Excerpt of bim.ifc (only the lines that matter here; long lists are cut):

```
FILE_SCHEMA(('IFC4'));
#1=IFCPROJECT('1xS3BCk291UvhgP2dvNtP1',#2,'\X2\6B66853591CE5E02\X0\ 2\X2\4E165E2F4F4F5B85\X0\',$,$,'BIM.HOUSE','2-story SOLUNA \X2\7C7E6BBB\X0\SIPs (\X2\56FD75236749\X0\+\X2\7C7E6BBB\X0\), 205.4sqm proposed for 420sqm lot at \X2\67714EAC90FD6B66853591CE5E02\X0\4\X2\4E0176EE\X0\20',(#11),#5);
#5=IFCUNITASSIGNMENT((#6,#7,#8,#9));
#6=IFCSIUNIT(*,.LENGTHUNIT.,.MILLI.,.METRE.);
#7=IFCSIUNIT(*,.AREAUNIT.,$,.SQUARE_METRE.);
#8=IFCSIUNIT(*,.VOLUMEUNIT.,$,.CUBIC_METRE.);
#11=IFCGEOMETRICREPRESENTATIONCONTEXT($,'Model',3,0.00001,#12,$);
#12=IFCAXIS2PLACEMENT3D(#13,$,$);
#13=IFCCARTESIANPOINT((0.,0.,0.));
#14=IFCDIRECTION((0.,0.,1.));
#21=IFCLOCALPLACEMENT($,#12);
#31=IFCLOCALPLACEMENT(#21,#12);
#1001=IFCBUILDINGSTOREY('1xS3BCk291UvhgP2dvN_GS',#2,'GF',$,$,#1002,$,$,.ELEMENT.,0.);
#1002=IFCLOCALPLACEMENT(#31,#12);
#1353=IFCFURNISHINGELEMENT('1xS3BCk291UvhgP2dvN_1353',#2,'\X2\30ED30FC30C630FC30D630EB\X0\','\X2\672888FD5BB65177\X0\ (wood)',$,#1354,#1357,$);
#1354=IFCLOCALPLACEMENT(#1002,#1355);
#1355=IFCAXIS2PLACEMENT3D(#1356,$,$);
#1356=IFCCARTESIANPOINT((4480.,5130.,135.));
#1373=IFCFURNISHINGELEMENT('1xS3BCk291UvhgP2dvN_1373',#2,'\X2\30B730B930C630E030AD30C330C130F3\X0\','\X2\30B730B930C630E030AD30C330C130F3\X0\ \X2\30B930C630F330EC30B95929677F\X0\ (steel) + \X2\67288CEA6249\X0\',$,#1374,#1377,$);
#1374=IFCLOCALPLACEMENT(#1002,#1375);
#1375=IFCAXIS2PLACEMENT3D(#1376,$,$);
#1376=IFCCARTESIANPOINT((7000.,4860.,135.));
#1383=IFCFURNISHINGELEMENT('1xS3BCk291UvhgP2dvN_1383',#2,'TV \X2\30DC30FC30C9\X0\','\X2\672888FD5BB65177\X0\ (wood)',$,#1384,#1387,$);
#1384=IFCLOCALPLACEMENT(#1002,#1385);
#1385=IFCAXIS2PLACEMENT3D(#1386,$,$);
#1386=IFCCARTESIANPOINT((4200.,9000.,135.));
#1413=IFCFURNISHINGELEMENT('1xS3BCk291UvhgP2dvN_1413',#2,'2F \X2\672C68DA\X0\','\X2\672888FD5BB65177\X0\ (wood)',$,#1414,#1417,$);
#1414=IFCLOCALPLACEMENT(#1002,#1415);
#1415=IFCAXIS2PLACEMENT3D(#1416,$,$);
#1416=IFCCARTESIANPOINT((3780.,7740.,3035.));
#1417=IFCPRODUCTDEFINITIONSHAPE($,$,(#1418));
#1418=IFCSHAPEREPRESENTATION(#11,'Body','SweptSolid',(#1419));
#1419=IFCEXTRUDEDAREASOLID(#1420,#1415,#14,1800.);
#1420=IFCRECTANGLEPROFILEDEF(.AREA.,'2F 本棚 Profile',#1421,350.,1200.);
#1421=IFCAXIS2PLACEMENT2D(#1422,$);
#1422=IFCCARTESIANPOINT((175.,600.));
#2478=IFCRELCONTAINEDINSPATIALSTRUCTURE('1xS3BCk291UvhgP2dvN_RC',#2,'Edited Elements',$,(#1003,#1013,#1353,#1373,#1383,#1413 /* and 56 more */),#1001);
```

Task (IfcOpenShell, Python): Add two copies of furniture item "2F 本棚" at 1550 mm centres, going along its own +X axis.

```python
import ifcopenshell
import ifcopenshell.api.geometry
import ifcopenshell.api.root
import ifcopenshell.util.element
import ifcopenshell.util.placement
import ifcopenshell.util.unit

model = ifcopenshell.open("bim.ifc")
unit_scale = ifcopenshell.util.unit.calculate_unit_scale(model)


def reuse_history(source, copy):
    """copy_class also copies each property set's owner history, people and application; keep the originals."""
    for rel in copy.IsDefinedBy:
        if rel.is_a("IfcRelDefinesByProperties") and (history := rel.RelatingPropertyDefinition.OwnerHistory):
            rel.RelatingPropertyDefinition.OwnerHistory = source.OwnerHistory
            ifcopenshell.util.element.remove_deep2(model, history)


source = model.by_guid("1xS3BCk291UvhgP2dvN_1413")
base = ifcopenshell.util.placement.get_local_placement(source.ObjectPlacement)
step = base[:3, 0] * 1.55 / unit_scale

for i in range(1, 3):
    copy = ifcopenshell.api.root.copy_class(model, product=source)
    copy.Representation = ifcopenshell.util.element.copy_deep(
        model, source.Representation, exclude=["IfcGeometricRepresentationContext", "IfcRepresentationMap"]
    )
    reuse_history(source, copy)
    matrix = base.copy()
    matrix[:3, 3] += i * step
    print("added at", matrix[:3, 3].round(3) + 0.0)
    ifcopenshell.api.geometry.edit_object_placement(model, product=copy, matrix=matrix, is_si=False)

model.write("bim_v2.ifc")
```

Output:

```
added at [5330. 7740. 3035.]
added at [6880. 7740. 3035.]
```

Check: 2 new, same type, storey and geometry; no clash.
